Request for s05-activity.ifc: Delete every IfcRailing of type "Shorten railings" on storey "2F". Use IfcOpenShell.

First a look at what the model holds.

```python
import ifcopenshell
import ifcopenshell.util.element

model = ifcopenshell.open("s05-activity.ifc")
print(model.schema)
storey = next(s for s in model.by_type("IfcBuildingStorey") if s.Name == "2F")
railings = [e for e in ifcopenshell.util.element.get_decomposition(storey) if e.is_a("IfcRailing")]
seen = {}
for e in railings:
    element_type = ifcopenshell.util.element.get_type(e)
    name = element_type.Name if element_type not in (None, e) else None
    seen[name] = seen.get(name, 0) + 1
for name, count in sorted(seen.items(), key=str):
    print(count, "x", name)
```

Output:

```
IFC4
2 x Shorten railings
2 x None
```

```python
import ifcopenshell
import ifcopenshell.api.root
import ifcopenshell.util.element

model = ifcopenshell.open("s05-activity.ifc")

storey = next(s for s in model.by_type("IfcBuildingStorey") if s.Name == "2F")
railings = [e for e in ifcopenshell.util.element.get_decomposition(storey) if e.is_a("IfcRailing")]
targets = [e for e in railings if (t := ifcopenshell.util.element.get_type(e)) not in (None, e) and t.Name == "Shorten railings"]

for e in targets:
    ifcopenshell.api.root.remove_product(model, product=e)
print(len(targets), "removed")

model.write("s05-activity_rev.ifc")
```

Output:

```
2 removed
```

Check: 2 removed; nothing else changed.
